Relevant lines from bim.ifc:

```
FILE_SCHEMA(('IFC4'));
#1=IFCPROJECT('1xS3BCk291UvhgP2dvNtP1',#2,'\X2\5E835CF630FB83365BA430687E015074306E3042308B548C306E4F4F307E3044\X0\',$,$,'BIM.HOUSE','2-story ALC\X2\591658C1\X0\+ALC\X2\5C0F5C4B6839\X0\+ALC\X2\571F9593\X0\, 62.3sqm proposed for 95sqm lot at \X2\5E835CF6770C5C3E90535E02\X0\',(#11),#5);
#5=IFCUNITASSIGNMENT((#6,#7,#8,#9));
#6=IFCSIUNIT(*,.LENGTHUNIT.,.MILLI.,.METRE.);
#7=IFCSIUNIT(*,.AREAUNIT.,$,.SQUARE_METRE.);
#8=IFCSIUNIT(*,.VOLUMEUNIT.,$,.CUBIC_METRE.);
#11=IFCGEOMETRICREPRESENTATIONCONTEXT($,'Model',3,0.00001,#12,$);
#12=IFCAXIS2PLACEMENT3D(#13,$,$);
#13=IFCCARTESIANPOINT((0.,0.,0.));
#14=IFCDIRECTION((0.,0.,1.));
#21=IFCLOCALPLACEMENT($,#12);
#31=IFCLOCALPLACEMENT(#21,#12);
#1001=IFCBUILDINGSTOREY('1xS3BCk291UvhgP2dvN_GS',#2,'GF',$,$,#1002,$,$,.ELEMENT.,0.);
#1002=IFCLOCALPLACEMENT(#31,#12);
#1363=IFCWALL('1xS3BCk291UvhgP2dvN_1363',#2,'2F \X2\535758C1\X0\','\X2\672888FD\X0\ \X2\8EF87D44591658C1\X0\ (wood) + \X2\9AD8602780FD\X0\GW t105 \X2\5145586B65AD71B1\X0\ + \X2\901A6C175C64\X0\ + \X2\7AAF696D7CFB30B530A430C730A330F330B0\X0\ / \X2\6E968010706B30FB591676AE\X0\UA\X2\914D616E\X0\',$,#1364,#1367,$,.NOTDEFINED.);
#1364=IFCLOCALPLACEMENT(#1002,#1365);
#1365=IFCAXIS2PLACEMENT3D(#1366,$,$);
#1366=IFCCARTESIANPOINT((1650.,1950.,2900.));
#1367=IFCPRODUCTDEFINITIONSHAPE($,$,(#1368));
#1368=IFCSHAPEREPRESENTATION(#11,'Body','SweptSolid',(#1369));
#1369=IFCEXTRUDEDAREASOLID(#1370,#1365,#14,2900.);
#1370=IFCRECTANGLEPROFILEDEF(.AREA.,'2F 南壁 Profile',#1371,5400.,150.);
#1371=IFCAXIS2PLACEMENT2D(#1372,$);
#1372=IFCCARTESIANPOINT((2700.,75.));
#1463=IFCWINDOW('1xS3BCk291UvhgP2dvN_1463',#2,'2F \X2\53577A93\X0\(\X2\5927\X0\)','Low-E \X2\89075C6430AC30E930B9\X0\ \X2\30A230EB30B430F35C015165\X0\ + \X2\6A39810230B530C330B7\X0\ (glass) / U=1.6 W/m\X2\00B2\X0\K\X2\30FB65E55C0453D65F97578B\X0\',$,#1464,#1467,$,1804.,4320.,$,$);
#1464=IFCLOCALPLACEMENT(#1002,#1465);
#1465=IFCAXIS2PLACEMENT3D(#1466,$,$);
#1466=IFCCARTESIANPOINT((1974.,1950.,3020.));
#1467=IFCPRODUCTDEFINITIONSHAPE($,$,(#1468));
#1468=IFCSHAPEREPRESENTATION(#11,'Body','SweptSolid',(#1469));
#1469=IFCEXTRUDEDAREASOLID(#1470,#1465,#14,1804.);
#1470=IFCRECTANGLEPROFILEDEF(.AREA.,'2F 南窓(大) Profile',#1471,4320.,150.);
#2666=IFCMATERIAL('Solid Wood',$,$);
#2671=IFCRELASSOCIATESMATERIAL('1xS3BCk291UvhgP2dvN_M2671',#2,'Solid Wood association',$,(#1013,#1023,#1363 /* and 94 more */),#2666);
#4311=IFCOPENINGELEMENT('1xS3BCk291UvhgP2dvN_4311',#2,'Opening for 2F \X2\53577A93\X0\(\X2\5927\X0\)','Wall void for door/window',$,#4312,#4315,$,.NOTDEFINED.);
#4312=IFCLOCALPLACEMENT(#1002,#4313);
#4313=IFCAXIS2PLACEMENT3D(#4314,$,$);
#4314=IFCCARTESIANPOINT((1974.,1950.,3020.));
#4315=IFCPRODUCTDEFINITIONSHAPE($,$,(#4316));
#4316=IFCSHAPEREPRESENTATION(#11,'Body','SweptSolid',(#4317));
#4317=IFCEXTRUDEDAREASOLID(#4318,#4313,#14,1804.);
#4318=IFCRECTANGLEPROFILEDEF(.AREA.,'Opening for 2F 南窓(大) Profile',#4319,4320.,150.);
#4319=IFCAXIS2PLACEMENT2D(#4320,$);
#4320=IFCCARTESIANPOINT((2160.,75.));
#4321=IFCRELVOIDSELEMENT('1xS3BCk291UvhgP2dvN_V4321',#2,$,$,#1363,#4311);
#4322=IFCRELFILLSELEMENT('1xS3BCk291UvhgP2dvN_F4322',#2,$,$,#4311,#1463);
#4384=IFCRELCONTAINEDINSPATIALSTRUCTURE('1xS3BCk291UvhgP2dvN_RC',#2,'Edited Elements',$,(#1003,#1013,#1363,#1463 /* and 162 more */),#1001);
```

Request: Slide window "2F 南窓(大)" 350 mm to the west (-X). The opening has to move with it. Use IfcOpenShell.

```python
import ifcopenshell
import ifcopenshell.api.geometry
import ifcopenshell.util.placement
import ifcopenshell.util.unit

model = ifcopenshell.open("bim.ifc")
unit_scale = ifcopenshell.util.unit.calculate_unit_scale(model)

window = model.by_id(1463)
opening = window.FillsVoids[0].RelatingOpeningElement
wall = opening.VoidsElements[0].RelatingBuildingElement

wall_matrix = ifcopenshell.util.placement.get_local_placement(wall.ObjectPlacement)
shift = wall_matrix[:3, 0] * -0.35 / unit_scale
before = ifcopenshell.util.placement.get_local_placement(window.ObjectPlacement)[:3, 3].copy()

# The window is not placed relative to its opening, so move both.
for product in (opening, window):
    matrix = ifcopenshell.util.placement.get_local_placement(product.ObjectPlacement)
    matrix[:3, 3] += shift
    ifcopenshell.api.geometry.edit_object_placement(model, product=product, matrix=matrix, is_si=False)

after = ifcopenshell.util.placement.get_local_placement(window.ObjectPlacement)[:3, 3]
print("window moved by", (after - before).round(3) + 0.0)

model.write("bim_updated.ifc")
```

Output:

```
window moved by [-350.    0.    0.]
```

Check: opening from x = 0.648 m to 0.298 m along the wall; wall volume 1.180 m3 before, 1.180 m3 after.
